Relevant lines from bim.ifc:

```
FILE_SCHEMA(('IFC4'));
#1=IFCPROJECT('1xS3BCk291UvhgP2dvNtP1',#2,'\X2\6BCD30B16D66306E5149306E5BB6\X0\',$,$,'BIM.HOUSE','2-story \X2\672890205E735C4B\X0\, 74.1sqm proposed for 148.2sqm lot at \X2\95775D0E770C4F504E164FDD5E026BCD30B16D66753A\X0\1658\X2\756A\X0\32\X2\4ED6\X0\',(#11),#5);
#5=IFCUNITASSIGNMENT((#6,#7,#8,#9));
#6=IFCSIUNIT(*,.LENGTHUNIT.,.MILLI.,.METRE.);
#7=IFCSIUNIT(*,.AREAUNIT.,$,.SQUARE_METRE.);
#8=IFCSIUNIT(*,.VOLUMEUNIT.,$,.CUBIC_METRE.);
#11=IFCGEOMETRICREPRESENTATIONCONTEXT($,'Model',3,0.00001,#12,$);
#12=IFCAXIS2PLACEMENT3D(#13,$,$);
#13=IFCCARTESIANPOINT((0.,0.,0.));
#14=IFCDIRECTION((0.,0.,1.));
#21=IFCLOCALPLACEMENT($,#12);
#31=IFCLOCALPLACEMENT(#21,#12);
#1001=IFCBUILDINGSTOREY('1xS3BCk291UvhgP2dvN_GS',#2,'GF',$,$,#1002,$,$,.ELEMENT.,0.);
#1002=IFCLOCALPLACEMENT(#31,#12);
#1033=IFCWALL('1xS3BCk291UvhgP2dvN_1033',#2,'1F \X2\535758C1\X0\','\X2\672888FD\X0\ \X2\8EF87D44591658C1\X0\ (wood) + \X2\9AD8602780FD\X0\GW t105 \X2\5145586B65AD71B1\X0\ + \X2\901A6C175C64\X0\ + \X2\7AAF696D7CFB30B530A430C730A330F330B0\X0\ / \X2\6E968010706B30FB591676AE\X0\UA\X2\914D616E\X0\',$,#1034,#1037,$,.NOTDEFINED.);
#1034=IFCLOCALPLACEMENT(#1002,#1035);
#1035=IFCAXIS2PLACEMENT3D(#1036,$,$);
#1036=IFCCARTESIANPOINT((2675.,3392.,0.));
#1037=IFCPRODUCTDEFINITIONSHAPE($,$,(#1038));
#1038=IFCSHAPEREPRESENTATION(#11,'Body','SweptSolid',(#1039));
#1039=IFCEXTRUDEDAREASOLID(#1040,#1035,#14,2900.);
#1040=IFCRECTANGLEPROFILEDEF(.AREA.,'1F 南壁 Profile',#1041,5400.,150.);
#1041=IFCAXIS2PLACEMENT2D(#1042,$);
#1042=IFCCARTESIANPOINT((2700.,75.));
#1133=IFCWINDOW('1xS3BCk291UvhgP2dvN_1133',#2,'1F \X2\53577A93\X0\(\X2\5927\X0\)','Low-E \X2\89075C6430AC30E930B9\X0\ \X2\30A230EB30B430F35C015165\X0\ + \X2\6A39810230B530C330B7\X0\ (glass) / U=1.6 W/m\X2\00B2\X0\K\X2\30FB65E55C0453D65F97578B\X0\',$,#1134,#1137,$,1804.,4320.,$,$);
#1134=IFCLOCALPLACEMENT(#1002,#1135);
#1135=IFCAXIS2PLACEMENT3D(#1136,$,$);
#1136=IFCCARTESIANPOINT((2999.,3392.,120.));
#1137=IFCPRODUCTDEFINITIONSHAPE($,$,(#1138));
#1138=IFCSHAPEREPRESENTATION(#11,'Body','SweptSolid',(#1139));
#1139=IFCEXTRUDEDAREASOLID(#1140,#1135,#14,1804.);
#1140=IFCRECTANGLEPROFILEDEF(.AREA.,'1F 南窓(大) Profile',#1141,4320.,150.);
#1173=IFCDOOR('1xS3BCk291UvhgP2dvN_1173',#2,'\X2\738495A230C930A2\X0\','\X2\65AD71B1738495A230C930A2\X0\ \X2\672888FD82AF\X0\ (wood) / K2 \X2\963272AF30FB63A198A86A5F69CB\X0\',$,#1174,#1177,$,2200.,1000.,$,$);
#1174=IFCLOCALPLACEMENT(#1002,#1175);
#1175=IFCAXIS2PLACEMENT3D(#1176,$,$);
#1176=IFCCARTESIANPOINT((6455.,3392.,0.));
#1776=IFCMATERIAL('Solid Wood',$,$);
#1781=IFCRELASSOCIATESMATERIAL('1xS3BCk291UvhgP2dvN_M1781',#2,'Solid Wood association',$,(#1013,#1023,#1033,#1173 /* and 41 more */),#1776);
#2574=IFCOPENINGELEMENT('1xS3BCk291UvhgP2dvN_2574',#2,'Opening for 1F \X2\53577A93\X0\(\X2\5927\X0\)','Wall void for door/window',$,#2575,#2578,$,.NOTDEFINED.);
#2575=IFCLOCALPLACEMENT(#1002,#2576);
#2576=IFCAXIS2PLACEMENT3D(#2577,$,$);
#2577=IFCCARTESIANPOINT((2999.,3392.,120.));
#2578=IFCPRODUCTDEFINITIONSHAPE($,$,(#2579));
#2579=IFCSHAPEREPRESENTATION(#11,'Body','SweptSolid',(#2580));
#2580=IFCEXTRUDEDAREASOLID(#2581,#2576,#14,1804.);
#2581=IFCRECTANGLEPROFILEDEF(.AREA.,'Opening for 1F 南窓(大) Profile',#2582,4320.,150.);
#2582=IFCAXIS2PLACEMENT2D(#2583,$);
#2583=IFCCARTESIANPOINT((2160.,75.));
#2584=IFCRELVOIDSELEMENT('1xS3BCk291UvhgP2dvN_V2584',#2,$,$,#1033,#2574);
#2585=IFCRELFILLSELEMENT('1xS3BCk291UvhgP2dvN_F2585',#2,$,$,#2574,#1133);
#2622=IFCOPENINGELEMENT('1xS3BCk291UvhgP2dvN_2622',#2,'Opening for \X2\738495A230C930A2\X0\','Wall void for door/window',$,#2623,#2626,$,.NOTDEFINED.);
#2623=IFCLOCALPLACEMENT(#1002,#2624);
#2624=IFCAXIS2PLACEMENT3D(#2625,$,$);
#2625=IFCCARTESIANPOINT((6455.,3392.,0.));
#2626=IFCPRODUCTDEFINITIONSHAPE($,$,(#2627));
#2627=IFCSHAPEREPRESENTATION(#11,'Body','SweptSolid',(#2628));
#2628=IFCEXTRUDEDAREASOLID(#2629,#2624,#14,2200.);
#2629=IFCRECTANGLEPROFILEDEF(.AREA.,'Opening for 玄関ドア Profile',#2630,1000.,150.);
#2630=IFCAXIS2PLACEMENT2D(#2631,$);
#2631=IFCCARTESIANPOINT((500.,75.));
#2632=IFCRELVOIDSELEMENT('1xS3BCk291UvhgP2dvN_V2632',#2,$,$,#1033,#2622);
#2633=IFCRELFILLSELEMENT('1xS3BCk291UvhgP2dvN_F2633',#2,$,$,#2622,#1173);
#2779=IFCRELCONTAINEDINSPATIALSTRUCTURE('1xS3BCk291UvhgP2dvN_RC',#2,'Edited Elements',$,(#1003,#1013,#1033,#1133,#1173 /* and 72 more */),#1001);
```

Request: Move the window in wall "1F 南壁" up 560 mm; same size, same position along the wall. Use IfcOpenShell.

```python
import numpy as np
import ifcopenshell
import ifcopenshell.api.geometry
import ifcopenshell.util.placement
import ifcopenshell.util.unit

model = ifcopenshell.open("bim.ifc")
unit_scale = ifcopenshell.util.unit.calculate_unit_scale(model)

window = model.by_guid("1xS3BCk291UvhgP2dvN_1133")
opening = window.FillsVoids[0].RelatingOpeningElement
dz = 0.56 / unit_scale

shift = np.array([0.0, 0.0, dz])
# The window is not placed relative to its opening, so move both.
for product in (opening, window):
    matrix = ifcopenshell.util.placement.get_local_placement(product.ObjectPlacement)
    matrix[:3, 3] += shift
    ifcopenshell.api.geometry.edit_object_placement(model, product=product, matrix=matrix, is_si=False)

print(f"moved by {dz * unit_scale:+.3f} m")

model.write("bim_updated.ifc")
```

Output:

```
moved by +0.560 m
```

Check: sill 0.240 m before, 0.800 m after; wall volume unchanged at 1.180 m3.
